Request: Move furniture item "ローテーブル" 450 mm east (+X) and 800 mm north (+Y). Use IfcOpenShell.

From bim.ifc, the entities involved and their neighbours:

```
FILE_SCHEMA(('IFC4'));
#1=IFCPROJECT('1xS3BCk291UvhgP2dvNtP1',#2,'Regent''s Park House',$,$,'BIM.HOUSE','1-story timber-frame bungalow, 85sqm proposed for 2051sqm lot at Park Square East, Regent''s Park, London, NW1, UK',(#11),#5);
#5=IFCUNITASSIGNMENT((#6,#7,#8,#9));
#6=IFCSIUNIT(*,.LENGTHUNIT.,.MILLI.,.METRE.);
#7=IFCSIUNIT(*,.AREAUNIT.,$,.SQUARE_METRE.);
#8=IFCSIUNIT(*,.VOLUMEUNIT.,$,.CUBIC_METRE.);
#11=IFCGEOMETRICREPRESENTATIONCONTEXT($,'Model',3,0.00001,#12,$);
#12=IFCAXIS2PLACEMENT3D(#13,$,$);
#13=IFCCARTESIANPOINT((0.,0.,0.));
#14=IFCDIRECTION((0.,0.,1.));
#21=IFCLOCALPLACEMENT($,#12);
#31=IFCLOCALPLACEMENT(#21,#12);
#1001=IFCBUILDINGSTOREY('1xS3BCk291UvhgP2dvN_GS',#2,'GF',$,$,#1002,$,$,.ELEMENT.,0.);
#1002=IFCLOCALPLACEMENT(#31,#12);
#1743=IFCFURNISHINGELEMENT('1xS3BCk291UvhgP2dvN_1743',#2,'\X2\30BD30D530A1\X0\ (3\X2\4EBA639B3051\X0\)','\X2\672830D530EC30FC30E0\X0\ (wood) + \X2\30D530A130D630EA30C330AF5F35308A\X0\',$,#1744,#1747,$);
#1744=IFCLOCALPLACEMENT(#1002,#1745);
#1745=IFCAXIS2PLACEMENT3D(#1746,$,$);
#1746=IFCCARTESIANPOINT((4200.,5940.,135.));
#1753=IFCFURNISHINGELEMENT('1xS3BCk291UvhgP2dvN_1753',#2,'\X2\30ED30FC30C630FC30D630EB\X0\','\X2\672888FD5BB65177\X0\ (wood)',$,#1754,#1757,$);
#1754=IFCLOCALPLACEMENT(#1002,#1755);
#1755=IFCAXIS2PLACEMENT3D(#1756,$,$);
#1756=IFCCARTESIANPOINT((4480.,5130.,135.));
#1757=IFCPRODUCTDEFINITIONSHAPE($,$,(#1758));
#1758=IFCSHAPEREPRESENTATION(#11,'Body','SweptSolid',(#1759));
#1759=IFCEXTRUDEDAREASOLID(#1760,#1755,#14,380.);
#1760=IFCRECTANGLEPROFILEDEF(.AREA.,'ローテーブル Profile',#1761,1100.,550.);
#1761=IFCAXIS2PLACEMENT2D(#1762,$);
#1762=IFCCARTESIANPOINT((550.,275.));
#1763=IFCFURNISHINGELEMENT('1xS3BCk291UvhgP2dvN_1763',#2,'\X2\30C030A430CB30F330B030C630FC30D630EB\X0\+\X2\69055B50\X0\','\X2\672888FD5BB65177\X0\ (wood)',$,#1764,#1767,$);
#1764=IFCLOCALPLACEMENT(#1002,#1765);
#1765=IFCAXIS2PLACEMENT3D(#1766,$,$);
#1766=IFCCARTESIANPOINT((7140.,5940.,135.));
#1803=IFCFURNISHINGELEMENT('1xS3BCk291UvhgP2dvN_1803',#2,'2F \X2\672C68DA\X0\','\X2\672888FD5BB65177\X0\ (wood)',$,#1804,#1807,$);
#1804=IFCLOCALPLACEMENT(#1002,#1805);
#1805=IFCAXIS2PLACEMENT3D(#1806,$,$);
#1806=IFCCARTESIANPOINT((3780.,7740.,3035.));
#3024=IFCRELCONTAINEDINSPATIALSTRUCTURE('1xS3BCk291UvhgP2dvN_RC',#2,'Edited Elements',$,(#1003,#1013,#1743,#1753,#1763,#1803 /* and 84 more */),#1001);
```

```python
import ifcopenshell
import ifcopenshell.api.geometry
import ifcopenshell.util.placement

model = ifcopenshell.open("bim.ifc")

item = model.by_guid("1xS3BCk291UvhgP2dvN_1753")
matrix = ifcopenshell.util.placement.get_local_placement(item.ObjectPlacement)
matrix[0, 3] += 450.0
matrix[1, 3] += 800.0
ifcopenshell.api.geometry.edit_object_placement(model, product=item, matrix=matrix, is_si=False)

print(ifcopenshell.util.placement.get_local_placement(item.ObjectPlacement).round(3) + 0.0)

model.write("bim_updated.ifc")
```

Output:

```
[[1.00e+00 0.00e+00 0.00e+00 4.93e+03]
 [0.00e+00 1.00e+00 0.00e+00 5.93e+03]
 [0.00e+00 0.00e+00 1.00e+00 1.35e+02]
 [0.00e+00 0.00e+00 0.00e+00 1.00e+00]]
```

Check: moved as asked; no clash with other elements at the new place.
